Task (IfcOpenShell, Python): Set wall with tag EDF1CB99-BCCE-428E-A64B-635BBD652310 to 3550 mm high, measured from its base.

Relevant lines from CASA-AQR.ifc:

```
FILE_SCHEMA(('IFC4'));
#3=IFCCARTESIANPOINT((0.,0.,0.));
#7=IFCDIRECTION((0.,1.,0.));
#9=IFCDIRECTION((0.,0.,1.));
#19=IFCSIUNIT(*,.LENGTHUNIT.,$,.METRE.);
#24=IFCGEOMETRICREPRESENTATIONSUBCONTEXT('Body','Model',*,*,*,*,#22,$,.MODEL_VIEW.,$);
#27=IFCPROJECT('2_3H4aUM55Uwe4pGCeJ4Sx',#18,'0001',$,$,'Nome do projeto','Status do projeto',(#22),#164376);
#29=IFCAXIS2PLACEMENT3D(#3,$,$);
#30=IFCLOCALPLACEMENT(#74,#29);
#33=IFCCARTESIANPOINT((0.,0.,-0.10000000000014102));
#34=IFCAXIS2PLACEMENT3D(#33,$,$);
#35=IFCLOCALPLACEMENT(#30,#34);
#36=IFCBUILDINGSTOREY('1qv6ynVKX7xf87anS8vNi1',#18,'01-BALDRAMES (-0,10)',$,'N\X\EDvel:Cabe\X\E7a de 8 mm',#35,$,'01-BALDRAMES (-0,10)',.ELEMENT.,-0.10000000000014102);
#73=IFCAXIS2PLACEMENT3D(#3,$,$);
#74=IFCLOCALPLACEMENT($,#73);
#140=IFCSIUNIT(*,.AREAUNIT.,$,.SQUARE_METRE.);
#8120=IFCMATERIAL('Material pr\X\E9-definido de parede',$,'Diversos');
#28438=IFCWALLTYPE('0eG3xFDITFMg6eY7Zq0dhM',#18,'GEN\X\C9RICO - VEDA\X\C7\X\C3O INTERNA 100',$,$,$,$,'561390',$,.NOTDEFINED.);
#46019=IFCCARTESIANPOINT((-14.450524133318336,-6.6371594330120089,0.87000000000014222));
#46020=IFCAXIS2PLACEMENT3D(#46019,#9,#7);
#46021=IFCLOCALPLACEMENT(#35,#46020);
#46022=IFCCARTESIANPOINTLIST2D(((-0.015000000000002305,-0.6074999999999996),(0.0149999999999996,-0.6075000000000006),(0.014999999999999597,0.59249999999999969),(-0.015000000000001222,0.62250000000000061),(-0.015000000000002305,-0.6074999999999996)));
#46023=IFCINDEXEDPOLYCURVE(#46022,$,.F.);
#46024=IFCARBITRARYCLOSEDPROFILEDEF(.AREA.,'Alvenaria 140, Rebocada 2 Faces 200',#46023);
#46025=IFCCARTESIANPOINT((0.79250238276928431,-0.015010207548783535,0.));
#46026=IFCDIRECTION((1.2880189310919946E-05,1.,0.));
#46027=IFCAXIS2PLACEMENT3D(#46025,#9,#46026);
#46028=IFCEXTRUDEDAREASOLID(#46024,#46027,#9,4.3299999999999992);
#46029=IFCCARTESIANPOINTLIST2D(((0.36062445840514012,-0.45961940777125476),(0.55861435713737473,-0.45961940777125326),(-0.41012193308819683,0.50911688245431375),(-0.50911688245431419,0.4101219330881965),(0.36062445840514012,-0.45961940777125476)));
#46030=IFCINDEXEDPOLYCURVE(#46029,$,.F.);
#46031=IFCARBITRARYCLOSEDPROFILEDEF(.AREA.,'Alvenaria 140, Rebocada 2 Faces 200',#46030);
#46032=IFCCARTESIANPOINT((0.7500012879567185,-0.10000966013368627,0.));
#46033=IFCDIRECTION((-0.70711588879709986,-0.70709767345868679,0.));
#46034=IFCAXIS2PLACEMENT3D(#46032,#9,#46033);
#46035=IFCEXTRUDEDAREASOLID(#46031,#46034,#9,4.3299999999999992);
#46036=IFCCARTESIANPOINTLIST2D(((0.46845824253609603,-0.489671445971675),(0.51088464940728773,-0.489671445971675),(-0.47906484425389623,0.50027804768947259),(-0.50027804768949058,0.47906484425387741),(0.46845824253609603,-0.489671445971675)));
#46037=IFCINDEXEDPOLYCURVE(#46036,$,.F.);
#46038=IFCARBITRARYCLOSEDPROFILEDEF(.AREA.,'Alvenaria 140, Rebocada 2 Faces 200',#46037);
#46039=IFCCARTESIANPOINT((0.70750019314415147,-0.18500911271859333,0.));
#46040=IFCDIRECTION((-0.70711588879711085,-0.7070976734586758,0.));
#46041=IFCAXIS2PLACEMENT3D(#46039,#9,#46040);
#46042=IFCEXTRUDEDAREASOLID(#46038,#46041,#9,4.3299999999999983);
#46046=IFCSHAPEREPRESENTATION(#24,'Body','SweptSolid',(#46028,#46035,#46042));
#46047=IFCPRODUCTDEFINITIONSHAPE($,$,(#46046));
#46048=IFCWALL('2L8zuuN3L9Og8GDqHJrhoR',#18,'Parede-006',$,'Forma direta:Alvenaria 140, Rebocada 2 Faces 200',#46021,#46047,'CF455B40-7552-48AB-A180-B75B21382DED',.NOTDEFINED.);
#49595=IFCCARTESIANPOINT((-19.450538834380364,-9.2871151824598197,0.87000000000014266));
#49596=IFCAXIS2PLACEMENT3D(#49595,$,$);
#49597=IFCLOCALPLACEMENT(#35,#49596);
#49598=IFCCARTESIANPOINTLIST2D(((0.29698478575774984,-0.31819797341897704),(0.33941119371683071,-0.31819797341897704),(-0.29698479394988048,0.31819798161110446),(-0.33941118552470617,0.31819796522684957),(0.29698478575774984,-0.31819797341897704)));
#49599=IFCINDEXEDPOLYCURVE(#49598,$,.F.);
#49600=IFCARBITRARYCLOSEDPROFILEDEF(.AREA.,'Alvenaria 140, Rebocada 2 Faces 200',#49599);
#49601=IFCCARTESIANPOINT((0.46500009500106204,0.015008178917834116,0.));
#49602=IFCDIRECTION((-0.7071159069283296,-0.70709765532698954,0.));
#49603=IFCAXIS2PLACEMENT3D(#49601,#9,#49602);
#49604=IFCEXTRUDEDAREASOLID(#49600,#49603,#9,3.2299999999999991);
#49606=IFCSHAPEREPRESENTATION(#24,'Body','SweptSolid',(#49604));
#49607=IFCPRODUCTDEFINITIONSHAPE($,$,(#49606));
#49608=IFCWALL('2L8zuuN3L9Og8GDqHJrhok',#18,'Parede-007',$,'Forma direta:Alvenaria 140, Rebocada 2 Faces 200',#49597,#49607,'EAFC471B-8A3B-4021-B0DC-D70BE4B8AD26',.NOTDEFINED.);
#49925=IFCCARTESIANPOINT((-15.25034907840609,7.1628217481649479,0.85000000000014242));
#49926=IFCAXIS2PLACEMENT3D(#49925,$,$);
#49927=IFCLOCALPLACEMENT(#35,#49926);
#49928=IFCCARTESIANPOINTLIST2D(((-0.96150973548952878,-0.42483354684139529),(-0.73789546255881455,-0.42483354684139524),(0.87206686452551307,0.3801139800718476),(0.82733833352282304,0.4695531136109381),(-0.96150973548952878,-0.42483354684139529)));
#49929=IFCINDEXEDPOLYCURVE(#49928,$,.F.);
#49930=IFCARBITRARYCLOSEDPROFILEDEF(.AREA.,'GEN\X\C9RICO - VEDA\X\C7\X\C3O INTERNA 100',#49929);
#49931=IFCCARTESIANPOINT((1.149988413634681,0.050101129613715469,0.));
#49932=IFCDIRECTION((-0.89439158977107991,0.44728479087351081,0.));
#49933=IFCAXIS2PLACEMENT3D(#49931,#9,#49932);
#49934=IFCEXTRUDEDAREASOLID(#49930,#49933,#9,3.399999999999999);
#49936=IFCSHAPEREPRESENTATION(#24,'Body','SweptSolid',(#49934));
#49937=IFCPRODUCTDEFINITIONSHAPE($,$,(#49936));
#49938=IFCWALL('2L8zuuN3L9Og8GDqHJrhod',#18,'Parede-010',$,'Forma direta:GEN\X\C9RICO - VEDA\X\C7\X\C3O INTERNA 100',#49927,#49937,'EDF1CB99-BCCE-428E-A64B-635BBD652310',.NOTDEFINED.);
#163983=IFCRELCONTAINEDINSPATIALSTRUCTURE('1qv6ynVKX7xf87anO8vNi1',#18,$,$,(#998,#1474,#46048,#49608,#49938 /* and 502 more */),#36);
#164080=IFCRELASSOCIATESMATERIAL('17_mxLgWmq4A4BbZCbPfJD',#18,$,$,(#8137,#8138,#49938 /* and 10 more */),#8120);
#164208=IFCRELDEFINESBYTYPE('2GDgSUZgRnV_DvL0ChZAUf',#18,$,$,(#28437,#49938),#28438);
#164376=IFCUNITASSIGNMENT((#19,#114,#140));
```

```python
import ifcopenshell
import ifcopenshell.geom
import ifcopenshell.util.representation
import ifcopenshell.util.shape
import ifcopenshell.util.unit

model = ifcopenshell.open("CASA-AQR.ifc")
unit_scale = ifcopenshell.util.unit.calculate_unit_scale(model)
settings = ifcopenshell.geom.settings()


def volume(element):
    """Net volume in cubic metres, openings subtracted."""
    shape = ifcopenshell.geom.create_shape(settings, element)
    return ifcopenshell.util.shape.get_volume(shape.geometry)


wall = model.by_guid("2L8zuuN3L9Og8GDqHJrhod")
before = volume(wall)

body = ifcopenshell.util.representation.get_representation(wall, "Model", "Body")
solid = body.Items[0]
old_height = solid.Depth
solid.Depth = 3.55 / unit_scale
after = volume(wall)

print(f"height {old_height:g} -> {solid.Depth:g}, volume {before:.3f} -> {after:.3f} m3")

model.write("CASA-AQR-out.ifc")
```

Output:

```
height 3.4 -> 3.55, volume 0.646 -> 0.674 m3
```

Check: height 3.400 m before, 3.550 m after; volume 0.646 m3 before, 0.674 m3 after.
